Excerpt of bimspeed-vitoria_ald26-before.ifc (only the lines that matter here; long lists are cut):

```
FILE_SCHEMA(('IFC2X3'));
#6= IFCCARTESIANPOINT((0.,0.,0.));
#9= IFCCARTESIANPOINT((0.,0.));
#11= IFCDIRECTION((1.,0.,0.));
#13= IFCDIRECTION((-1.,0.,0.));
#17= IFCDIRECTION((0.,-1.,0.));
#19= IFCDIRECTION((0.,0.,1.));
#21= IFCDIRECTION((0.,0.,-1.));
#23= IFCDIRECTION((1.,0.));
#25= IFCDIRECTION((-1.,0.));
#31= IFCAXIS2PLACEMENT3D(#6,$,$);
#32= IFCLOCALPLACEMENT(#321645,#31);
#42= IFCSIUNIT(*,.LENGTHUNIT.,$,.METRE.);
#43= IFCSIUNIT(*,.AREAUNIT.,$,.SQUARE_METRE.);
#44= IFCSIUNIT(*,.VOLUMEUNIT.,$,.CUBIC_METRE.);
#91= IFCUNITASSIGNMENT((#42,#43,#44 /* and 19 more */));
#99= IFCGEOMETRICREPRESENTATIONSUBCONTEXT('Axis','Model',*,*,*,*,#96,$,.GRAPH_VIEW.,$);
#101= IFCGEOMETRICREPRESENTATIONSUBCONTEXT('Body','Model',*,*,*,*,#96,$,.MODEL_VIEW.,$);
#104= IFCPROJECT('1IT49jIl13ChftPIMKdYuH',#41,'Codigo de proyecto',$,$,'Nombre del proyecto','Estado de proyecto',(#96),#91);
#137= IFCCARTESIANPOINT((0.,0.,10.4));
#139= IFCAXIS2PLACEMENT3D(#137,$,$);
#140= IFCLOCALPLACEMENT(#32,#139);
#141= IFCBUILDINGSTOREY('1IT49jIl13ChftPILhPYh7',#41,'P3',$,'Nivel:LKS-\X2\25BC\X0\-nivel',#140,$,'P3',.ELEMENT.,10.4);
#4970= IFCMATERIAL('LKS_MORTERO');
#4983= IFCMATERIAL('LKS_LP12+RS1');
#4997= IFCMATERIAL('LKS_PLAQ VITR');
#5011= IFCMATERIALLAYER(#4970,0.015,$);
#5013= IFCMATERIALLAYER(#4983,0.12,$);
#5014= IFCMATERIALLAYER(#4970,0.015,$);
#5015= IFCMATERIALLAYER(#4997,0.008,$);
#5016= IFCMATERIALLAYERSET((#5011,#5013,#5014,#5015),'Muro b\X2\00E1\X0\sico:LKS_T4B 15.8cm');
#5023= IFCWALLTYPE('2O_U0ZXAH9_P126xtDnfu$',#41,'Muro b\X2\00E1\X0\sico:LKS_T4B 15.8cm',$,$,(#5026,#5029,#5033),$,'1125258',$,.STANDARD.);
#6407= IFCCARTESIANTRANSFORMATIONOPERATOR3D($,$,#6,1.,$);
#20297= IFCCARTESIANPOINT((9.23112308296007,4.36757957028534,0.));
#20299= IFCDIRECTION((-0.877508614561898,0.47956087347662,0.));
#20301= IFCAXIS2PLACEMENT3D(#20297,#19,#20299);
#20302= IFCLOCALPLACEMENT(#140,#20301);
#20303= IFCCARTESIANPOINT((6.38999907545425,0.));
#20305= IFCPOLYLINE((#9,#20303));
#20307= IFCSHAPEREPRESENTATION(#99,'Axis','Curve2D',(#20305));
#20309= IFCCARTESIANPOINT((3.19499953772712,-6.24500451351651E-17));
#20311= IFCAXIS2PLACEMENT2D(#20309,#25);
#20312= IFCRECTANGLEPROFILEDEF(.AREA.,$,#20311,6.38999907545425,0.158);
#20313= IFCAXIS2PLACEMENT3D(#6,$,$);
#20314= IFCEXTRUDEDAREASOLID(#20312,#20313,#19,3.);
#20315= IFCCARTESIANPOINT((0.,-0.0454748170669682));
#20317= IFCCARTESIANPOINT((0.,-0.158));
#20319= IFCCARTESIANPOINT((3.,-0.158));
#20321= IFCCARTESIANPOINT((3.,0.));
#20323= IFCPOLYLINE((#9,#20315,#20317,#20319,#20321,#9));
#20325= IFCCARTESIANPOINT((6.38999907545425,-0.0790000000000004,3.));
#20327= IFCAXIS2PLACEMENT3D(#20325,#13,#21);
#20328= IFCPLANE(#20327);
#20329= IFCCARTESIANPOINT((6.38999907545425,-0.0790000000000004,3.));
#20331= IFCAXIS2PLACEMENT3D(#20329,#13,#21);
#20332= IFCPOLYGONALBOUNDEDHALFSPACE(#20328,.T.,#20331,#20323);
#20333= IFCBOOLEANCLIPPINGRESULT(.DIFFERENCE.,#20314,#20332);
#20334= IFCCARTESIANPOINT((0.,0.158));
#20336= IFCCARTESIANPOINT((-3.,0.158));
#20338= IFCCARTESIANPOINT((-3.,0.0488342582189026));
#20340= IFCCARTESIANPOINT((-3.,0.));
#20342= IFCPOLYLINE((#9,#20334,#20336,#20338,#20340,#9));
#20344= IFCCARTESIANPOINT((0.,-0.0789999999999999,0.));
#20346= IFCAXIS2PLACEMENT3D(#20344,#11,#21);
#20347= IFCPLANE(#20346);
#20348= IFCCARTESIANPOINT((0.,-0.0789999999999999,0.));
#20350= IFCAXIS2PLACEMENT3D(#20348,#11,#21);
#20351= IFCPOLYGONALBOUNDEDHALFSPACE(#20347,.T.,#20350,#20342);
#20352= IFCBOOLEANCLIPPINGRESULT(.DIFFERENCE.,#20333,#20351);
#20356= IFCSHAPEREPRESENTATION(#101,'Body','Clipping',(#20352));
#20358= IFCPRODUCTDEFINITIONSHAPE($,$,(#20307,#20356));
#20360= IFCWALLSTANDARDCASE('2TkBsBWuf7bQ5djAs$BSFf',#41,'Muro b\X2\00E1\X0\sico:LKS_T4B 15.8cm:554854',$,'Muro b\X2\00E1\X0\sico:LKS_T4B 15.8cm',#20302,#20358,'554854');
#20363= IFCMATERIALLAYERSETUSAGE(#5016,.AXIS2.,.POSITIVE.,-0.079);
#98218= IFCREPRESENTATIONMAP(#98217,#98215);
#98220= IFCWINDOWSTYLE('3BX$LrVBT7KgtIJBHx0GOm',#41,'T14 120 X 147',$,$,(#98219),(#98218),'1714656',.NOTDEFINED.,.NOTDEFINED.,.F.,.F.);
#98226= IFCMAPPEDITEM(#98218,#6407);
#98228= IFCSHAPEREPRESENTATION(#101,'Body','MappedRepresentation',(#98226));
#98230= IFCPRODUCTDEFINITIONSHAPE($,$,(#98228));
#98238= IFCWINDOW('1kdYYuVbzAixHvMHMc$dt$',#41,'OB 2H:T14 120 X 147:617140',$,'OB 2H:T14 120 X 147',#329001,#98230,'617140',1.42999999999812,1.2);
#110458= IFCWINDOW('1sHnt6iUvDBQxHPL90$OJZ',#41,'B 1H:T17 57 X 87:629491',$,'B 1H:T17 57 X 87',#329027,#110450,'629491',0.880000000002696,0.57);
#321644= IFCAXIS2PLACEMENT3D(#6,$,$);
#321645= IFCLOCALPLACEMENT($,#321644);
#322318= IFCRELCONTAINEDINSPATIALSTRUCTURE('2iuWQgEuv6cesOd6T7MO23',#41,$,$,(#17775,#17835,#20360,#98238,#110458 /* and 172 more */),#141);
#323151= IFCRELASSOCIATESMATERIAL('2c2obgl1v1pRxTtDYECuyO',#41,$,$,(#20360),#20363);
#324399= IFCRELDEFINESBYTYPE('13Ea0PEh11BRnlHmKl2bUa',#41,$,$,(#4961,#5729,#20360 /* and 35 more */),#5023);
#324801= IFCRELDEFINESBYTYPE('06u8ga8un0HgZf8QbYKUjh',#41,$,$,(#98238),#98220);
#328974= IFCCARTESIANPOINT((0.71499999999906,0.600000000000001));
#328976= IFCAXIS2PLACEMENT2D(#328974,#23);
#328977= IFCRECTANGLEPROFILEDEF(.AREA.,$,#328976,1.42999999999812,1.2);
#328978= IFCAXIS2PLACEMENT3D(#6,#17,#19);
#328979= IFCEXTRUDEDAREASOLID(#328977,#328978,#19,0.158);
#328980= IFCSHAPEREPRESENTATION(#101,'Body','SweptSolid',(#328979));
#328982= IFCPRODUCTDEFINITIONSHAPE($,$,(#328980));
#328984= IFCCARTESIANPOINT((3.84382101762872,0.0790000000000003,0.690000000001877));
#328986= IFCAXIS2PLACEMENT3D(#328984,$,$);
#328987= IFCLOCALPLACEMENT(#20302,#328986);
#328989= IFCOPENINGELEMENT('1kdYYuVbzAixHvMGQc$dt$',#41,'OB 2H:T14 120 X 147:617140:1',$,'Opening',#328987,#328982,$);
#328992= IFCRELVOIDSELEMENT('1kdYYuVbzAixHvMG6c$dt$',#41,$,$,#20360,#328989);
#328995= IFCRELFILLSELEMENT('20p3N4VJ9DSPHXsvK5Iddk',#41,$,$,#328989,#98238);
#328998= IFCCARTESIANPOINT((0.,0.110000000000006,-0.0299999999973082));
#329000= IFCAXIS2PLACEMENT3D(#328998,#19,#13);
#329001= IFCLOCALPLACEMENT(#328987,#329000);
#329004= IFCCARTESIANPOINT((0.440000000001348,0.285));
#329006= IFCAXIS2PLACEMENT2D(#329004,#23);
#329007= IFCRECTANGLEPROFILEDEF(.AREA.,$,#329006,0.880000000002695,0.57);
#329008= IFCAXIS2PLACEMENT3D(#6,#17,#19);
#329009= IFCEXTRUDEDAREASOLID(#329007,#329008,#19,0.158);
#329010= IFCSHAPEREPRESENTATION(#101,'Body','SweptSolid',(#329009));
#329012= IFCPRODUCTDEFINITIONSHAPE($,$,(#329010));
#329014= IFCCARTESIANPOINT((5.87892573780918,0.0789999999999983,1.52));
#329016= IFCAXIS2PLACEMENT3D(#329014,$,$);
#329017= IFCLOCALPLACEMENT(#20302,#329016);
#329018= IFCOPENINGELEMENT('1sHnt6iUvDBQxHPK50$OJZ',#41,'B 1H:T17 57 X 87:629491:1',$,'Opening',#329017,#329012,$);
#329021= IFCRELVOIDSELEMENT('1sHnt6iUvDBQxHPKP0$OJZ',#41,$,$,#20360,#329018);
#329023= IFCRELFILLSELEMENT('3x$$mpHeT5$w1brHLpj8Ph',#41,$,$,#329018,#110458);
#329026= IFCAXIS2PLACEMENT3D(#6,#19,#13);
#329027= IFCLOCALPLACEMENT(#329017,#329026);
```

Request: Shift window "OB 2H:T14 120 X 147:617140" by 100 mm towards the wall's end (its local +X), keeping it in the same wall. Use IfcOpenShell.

```python
import ifcopenshell
import ifcopenshell.api.geometry
import ifcopenshell.util.placement
import ifcopenshell.util.unit

model = ifcopenshell.open("bimspeed-vitoria_ald26-before.ifc")
unit_scale = ifcopenshell.util.unit.calculate_unit_scale(model)

window = model.by_guid("1kdYYuVbzAixHvMHMc$dt$")
opening = window.FillsVoids[0].RelatingOpeningElement
wall = opening.VoidsElements[0].RelatingBuildingElement

wall_matrix = ifcopenshell.util.placement.get_local_placement(wall.ObjectPlacement)
shift = wall_matrix[:3, 0] * 0.1 / unit_scale
before = ifcopenshell.util.placement.get_local_placement(window.ObjectPlacement)[:3, 3].copy()

# The window is placed relative to its opening, so it follows when the opening moves.
matrix = ifcopenshell.util.placement.get_local_placement(opening.ObjectPlacement)
matrix[:3, 3] += shift
ifcopenshell.api.geometry.edit_object_placement(
    model, product=opening, matrix=matrix, is_si=False, should_transform_children=True
)

after = ifcopenshell.util.placement.get_local_placement(window.ObjectPlacement)[:3, 3]
print("window moved by", (after - before).round(3) + 0.0)

model.write("bimspeed-vitoria_ald26-before_rev.ifc")
```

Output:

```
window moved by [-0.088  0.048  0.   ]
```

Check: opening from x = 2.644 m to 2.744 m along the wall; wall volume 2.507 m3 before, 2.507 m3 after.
